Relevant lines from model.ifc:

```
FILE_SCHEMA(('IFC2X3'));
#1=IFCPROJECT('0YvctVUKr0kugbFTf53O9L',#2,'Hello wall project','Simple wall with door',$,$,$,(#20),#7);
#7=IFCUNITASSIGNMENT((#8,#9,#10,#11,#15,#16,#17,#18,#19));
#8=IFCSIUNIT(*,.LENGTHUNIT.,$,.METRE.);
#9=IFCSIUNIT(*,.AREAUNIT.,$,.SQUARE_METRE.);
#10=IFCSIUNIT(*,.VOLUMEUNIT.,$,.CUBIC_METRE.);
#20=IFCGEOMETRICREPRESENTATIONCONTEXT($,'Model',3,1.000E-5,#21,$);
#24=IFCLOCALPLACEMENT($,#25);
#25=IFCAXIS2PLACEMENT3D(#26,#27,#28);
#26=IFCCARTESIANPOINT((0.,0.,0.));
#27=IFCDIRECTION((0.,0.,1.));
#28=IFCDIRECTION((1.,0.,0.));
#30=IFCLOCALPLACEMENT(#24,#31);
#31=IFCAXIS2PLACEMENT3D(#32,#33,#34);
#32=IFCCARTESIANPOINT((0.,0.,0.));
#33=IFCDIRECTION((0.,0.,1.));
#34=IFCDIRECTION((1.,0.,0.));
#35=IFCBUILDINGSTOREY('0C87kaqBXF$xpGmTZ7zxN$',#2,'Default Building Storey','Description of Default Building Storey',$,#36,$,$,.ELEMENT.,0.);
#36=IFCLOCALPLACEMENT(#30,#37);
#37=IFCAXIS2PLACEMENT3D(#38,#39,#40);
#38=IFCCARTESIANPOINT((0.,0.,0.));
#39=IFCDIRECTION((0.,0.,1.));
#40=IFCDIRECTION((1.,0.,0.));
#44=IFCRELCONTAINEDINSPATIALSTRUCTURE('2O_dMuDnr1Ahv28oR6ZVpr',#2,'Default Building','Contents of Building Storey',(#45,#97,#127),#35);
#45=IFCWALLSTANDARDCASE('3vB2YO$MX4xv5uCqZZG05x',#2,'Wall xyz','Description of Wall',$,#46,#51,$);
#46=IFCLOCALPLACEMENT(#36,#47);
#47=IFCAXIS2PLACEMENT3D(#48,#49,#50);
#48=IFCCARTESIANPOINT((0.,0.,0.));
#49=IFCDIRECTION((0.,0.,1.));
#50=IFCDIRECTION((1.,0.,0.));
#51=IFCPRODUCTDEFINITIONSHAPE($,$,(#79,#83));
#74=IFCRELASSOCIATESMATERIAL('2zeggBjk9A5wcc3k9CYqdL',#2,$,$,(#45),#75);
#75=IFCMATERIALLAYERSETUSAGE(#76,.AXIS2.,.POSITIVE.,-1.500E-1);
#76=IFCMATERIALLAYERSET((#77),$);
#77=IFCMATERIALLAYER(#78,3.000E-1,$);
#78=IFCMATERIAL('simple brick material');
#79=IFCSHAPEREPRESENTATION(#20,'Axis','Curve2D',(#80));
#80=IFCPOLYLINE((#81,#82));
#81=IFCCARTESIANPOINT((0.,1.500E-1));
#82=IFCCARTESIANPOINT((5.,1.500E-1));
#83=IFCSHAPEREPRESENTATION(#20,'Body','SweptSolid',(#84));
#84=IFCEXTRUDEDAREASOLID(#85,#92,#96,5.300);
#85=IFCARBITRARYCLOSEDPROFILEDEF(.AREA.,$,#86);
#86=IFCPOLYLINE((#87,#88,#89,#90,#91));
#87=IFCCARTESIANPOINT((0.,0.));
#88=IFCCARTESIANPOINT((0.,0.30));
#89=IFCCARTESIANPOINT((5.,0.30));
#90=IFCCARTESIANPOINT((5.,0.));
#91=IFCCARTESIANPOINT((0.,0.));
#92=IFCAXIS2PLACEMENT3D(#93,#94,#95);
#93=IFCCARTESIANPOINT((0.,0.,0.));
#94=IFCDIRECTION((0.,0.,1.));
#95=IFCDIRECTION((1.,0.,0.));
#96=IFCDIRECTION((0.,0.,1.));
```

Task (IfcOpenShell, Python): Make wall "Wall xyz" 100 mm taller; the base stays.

```python
import ifcopenshell
import ifcopenshell.geom
import ifcopenshell.util.shape
import ifcopenshell.util.unit

model = ifcopenshell.open("model.ifc")
unit_scale = ifcopenshell.util.unit.calculate_unit_scale(model)
settings = ifcopenshell.geom.settings()


def volume(element):
    """Net volume in cubic metres, openings subtracted."""
    shape = ifcopenshell.geom.create_shape(settings, element)
    return ifcopenshell.util.shape.get_volume(shape.geometry)


wall = model.by_guid("3vB2YO$MX4xv5uCqZZG05x")
before = volume(wall)

body = next(r for r in wall.Representation.Representations if r.RepresentationIdentifier == "Body")
solid = body.Items[0]
old_height = solid.Depth
solid.Depth += 0.1 / unit_scale
after = volume(wall)

print(f"height {old_height:g} -> {solid.Depth:g}, volume {before:.3f} -> {after:.3f} m3")

model.write("model_v2.ifc")
```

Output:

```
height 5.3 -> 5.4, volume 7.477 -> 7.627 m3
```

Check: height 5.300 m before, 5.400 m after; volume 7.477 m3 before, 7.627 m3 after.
